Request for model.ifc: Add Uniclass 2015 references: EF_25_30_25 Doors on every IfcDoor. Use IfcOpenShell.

First a look at what the model holds.

```python
import ifcopenshell

model = ifcopenshell.open("model.ifc")
print(model.schema)
print("classifications:", [c.Name for c in model.by_type("IfcClassification")])
for ifc_class in ("IfcDoor", "IfcRoof", "IfcStair", "IfcWall", "IfcWindow"):
    print(ifc_class, len(model.by_type(ifc_class)))
```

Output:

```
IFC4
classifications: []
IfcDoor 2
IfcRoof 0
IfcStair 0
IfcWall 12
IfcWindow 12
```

```python
import ifcopenshell
import ifcopenshell.api.classification

model = ifcopenshell.open("model.ifc")

system = ifcopenshell.api.classification.add_classification(model, classification="Uniclass 2015")

codes = {
    "IfcDoor": ("EF_25_30_25", "Doors"),
}
for ifc_class, (code, name) in codes.items():
    products = model.by_type(ifc_class)
    ifcopenshell.api.classification.add_reference(
        model, products=products, classification=system, identification=code, name=name
    )
    print(code, len(products))

model.write("model-out.ifc")
```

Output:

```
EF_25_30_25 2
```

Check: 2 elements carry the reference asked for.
